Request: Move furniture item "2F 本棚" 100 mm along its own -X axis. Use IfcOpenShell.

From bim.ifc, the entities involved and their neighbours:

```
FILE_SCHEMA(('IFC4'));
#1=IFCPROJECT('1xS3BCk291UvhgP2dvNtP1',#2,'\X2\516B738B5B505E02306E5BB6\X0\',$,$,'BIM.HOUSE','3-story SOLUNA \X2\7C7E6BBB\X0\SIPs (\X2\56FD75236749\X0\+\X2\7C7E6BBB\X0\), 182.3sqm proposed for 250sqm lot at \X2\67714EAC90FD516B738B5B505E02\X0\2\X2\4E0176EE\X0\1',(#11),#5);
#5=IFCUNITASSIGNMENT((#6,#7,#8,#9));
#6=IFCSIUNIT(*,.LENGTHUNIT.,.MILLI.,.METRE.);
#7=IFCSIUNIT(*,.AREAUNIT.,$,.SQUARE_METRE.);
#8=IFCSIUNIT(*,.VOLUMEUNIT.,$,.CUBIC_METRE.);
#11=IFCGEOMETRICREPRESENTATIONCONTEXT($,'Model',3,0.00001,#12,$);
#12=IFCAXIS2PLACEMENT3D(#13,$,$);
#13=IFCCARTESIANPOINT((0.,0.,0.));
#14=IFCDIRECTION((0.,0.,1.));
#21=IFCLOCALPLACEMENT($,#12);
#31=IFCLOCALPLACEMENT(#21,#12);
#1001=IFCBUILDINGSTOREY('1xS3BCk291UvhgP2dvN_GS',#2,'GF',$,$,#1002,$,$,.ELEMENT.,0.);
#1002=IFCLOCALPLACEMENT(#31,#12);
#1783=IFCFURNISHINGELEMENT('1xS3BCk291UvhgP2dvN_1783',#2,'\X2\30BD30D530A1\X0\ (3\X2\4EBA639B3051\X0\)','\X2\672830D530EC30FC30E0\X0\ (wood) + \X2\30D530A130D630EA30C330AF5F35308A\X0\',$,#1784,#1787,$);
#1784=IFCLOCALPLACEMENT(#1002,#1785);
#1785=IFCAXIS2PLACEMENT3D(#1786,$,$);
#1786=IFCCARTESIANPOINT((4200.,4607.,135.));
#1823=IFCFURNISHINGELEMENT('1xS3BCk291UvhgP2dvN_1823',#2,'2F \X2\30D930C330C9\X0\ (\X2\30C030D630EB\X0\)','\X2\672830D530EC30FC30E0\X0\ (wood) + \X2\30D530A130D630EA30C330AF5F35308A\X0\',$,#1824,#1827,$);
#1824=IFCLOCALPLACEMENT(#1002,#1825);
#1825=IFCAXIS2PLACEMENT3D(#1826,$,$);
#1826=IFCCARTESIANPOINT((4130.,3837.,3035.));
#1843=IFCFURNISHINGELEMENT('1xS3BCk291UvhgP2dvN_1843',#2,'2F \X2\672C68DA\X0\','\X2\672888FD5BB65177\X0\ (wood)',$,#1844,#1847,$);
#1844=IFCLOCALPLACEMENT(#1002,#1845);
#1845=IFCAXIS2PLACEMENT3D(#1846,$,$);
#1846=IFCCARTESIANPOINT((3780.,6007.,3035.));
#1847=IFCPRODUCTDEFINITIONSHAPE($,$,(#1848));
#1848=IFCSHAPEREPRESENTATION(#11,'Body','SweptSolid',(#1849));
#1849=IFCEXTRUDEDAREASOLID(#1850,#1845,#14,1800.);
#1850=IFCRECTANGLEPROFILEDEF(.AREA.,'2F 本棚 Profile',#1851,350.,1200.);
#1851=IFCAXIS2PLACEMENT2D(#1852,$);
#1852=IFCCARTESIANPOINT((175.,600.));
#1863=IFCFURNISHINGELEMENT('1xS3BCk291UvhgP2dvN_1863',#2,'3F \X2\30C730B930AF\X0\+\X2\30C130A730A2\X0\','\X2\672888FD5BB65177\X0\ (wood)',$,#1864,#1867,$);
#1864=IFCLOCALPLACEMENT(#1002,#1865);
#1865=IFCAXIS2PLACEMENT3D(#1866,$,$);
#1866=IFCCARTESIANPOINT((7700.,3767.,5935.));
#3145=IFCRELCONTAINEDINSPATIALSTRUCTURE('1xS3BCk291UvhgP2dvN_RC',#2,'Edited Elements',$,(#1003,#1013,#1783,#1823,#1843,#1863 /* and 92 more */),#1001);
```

```python
import ifcopenshell
import ifcopenshell.api.geometry
import ifcopenshell.util.placement
import ifcopenshell.util.unit

model = ifcopenshell.open("bim.ifc")
unit_scale = ifcopenshell.util.unit.calculate_unit_scale(model)

item = model.by_guid("1xS3BCk291UvhgP2dvN_1843")
matrix = ifcopenshell.util.placement.get_local_placement(item.ObjectPlacement)
matrix[:3, 3] -= matrix[:3, 0] * 0.1 / unit_scale
ifcopenshell.api.geometry.edit_object_placement(model, product=item, matrix=matrix, is_si=False)

print(ifcopenshell.util.placement.get_local_placement(item.ObjectPlacement).round(3) + 0.0)

model.write("bim_rev.ifc")
```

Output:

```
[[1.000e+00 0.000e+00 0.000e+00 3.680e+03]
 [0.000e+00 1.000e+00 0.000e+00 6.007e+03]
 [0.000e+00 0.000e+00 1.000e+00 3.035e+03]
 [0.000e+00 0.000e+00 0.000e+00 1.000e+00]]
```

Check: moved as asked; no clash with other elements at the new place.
